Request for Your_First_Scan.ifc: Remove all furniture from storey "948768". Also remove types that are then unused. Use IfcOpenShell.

First a look at what the model holds.

```python
import ifcopenshell
import ifcopenshell.util.element

model = ifcopenshell.open("Your_First_Scan.ifc")
print(model.schema)
storey = next(s for s in model.by_type("IfcBuildingStorey") if s.Name == "948768")
furniture = [e for e in ifcopenshell.util.element.get_decomposition(storey) if e.is_a("IfcFurnishingElement")]
seen = {}
for e in furniture:
    element_type = ifcopenshell.util.element.get_type(e)
    name = element_type.Name if element_type not in (None, e) else None
    seen[name] = seen.get(name, 0) + 1
for name, count in sorted(seen.items(), key=str):
    print(count, "x", name)
```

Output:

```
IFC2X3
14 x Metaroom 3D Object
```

```python
import ifcopenshell
import ifcopenshell.api.root
import ifcopenshell.util.element

model = ifcopenshell.open("Your_First_Scan.ifc")

storey = next(s for s in model.by_type("IfcBuildingStorey") if s.Name == "948768")
furniture = [e for e in ifcopenshell.util.element.get_decomposition(storey) if e.is_a("IfcFurnishingElement")]
types = {ifcopenshell.util.element.get_type(e) for e in furniture} - {None, *furniture}

for e in furniture:
    ifcopenshell.api.root.remove_product(model, product=e)
print(len(furniture), "removed")

unused = [t for t in types if not ifcopenshell.util.element.get_types(t)]
for t in unused:
    ifcopenshell.api.root.remove_product(model, product=t)
print(len(unused), "unused types removed")

model.write("Your_First_Scan_v2.ifc")
```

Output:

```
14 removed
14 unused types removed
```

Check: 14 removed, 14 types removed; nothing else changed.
